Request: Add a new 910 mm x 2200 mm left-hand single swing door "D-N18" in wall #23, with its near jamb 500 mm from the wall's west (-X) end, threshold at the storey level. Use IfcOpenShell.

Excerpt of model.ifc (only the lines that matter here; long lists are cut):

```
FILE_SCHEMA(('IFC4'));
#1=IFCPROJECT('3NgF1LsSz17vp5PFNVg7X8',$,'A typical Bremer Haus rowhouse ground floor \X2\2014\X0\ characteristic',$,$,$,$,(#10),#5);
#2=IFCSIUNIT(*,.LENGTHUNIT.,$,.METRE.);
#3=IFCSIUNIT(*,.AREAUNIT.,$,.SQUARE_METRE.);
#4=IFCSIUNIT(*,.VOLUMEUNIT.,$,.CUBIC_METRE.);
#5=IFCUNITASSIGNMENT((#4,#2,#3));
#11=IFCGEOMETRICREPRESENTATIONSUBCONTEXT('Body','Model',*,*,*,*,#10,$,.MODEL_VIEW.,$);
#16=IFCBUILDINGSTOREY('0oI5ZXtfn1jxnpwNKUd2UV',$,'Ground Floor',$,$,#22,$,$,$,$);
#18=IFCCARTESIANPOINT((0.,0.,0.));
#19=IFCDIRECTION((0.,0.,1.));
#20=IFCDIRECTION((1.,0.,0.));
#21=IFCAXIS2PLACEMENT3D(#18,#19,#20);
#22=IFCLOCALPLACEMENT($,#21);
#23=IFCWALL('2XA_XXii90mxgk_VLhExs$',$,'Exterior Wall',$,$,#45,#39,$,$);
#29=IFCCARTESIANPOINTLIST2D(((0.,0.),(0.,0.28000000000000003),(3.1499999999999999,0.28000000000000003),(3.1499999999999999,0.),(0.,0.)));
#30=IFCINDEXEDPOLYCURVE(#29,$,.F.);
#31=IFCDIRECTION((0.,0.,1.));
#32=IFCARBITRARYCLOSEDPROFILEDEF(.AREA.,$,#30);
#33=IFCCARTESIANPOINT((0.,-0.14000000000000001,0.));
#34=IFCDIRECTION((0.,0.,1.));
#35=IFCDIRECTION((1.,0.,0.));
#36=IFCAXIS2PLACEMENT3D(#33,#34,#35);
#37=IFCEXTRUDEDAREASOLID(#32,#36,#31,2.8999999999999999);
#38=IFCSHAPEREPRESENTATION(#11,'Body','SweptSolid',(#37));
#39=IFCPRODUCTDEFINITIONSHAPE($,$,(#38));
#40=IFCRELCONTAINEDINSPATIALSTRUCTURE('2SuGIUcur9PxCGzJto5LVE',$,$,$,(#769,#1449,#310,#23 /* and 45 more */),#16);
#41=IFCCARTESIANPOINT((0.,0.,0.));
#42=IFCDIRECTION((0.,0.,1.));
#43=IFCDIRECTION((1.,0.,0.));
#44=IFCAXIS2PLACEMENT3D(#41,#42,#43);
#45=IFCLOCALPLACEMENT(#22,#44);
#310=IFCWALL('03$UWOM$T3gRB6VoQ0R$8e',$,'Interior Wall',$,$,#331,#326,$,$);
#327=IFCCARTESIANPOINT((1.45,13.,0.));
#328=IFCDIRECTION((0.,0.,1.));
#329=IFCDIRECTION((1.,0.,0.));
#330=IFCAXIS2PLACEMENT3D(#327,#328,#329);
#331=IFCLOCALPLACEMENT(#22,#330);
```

```python
import numpy as np
import ifcopenshell
import ifcopenshell.api.feature
import ifcopenshell.api.geometry
import ifcopenshell.api.root
import ifcopenshell.api.spatial
import ifcopenshell.geom
import ifcopenshell.util.element
import ifcopenshell.util.placement
import ifcopenshell.util.representation
import ifcopenshell.util.shape
import ifcopenshell.util.unit

model = ifcopenshell.open("model.ifc")
unit_scale = ifcopenshell.util.unit.calculate_unit_scale(model)
settings = ifcopenshell.geom.settings()


def volume(element):
    """Net volume in cubic metres, openings subtracted."""
    shape = ifcopenshell.geom.create_shape(settings, element)
    return ifcopenshell.util.shape.get_volume(shape.geometry)


wall = model.by_guid("2XA_XXii90mxgk_VLhExs$")
storey = ifcopenshell.util.element.get_container(wall, ifc_class="IfcBuildingStorey")
context = ifcopenshell.util.representation.get_context(model, "Model", "Body", "MODEL_VIEW")
before = volume(wall)

width, height, from_end, sill = 0.91, 2.2, 0.5, 0.0  # metres

# The wall runs along its own X axis, and the end named is its -X end.
wall_shape = ifcopenshell.geom.create_shape(settings, wall)
x, y, z = ifcopenshell.util.shape.get_vertices(wall_shape.geometry).T
start = x.min() + from_end
face, thickness = float(y.min()), float(y.max() - y.min())
wall_matrix = ifcopenshell.util.placement.get_local_placement(wall.ObjectPlacement)
level = ifcopenshell.util.placement.get_local_placement(storey.ObjectPlacement)[2, 3]


def in_wall(x, y):
    """Placement at x, y metres in the wall's axes, at sill height."""
    matrix = wall_matrix.copy()
    matrix[:, 3] = wall_matrix @ np.array([x / unit_scale, y / unit_scale, 0.0, 1.0])
    matrix[2, 3] = level + sill / unit_scale
    return matrix


# Opening: a box that overshoots both wall faces by 50 mm.
opening = ifcopenshell.api.root.create_entity(model, ifc_class="IfcOpeningElement", predefined_type="OPENING")
box = ifcopenshell.api.geometry.add_wall_representation(
    model, context=context, length=width, height=height, thickness=thickness + 0.1
)
ifcopenshell.api.geometry.assign_representation(model, product=opening, representation=box)
ifcopenshell.api.geometry.edit_object_placement(model, product=opening, matrix=in_wall(start, face - 0.05), is_si=False)
ifcopenshell.api.feature.add_feature(model, feature=opening, element=wall)

door = ifcopenshell.api.root.create_entity(model, ifc_class="IfcDoor", name="D-N18", predefined_type="DOOR")
door.OverallWidth, door.OverallHeight = width / unit_scale, height / unit_scale
door.OperationType = "SINGLE_SWING_LEFT"
body = ifcopenshell.api.geometry.add_door_representation(
    model,
    context=context,
    overall_width=door.OverallWidth,
    overall_height=door.OverallHeight,
    operation_type="SINGLE_SWING_LEFT",
    lining_properties={"LiningDepth": thickness / unit_scale, "ThresholdDepth": thickness / unit_scale},
)
ifcopenshell.api.geometry.assign_representation(model, product=door, representation=body)
ifcopenshell.api.spatial.assign_container(model, products=[door], relating_structure=storey)
ifcopenshell.api.feature.add_filling(model, opening=opening, element=door)

# The lining spans the wall, so the door starts at the wall face.
ifcopenshell.api.geometry.edit_object_placement(model, product=door, matrix=in_wall(start, face), is_si=False)

after = volume(wall)

print(f"wall volume {before:.3f} -> {after:.3f} m3")

model.write("model_rev.ifc")
```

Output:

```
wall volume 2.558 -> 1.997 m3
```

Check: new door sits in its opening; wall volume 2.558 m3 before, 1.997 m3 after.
